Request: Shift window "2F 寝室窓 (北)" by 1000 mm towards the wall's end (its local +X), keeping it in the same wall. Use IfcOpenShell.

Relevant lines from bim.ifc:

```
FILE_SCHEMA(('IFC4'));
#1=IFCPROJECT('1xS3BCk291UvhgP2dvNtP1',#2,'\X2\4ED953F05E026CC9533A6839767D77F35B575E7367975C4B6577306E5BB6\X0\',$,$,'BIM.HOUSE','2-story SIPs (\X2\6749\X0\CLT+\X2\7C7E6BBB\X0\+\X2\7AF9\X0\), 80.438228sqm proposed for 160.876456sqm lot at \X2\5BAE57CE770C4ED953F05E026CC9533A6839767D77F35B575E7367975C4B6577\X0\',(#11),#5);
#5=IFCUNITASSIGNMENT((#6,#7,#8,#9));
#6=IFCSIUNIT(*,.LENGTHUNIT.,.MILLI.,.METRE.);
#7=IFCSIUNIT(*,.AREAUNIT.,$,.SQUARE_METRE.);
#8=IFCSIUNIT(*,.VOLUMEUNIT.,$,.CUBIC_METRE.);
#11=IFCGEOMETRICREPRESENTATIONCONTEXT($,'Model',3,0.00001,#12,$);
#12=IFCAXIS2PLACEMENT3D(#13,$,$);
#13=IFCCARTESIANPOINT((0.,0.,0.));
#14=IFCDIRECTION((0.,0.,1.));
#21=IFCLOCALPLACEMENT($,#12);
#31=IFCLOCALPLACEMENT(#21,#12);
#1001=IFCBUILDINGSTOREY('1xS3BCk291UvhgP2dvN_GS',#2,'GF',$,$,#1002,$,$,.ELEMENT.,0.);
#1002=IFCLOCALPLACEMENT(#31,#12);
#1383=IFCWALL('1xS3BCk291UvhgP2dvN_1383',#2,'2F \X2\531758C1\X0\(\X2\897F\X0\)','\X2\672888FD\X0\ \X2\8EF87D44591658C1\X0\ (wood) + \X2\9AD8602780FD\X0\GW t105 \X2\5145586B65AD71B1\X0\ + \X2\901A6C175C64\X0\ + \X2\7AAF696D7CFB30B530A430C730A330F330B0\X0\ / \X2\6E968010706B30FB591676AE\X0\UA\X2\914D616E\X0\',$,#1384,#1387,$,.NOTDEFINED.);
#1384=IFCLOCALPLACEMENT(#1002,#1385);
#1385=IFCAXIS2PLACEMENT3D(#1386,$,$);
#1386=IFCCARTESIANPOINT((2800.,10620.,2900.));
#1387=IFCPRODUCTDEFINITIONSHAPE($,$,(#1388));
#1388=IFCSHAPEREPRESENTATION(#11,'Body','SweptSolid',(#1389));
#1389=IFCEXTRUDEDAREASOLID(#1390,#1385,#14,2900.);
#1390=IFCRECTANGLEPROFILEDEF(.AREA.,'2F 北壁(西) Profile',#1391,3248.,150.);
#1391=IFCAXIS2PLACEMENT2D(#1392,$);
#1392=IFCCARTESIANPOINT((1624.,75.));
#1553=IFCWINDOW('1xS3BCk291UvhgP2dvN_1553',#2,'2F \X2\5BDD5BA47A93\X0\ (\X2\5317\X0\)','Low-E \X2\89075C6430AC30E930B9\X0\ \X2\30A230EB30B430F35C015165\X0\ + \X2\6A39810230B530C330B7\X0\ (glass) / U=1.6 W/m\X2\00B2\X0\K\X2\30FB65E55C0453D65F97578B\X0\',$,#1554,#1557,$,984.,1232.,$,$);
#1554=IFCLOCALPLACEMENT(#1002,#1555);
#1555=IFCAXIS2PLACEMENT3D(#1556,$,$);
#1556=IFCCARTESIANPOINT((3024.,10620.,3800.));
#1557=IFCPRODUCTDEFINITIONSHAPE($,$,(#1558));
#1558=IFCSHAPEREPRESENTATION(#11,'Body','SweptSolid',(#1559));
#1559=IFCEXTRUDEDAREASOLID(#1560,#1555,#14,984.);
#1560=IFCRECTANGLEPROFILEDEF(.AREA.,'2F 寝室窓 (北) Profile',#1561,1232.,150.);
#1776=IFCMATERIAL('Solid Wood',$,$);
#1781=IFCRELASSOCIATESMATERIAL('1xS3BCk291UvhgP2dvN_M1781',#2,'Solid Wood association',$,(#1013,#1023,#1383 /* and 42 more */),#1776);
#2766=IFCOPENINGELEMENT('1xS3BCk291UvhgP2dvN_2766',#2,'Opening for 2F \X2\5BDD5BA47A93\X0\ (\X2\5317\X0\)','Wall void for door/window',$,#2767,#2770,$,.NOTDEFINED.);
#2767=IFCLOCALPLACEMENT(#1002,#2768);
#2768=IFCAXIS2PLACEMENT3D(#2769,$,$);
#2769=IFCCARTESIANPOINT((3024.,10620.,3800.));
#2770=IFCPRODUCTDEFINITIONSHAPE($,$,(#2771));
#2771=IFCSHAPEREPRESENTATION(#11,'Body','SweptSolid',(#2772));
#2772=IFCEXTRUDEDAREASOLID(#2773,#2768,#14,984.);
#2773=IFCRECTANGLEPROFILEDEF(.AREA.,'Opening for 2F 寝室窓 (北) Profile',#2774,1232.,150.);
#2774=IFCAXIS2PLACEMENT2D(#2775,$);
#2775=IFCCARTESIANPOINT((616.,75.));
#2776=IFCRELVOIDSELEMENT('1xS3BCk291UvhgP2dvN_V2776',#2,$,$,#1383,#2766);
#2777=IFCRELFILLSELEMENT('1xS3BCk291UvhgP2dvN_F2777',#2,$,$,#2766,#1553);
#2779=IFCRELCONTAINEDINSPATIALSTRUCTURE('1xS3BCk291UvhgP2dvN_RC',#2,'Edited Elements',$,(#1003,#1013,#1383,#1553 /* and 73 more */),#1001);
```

```python
import ifcopenshell
import ifcopenshell.api.geometry
import ifcopenshell.util.placement

model = ifcopenshell.open("bim.ifc")

window = model.by_guid("1xS3BCk291UvhgP2dvN_1553")
opening = window.FillsVoids[0].RelatingOpeningElement
wall = opening.VoidsElements[0].RelatingBuildingElement

wall_matrix = ifcopenshell.util.placement.get_local_placement(wall.ObjectPlacement)
shift = wall_matrix[:3, 0] * 1000.0
before = ifcopenshell.util.placement.get_local_placement(window.ObjectPlacement)[:3, 3].copy()

# The window is not placed relative to its opening, so move both.
for product in (opening, window):
    matrix = ifcopenshell.util.placement.get_local_placement(product.ObjectPlacement)
    matrix[:3, 3] += shift
    ifcopenshell.api.geometry.edit_object_placement(model, product=product, matrix=matrix, is_si=False)

after = ifcopenshell.util.placement.get_local_placement(window.ObjectPlacement)[:3, 3]
print("window moved by", (after - before).round(3) + 0.0)

model.write("bim_rev.ifc")
```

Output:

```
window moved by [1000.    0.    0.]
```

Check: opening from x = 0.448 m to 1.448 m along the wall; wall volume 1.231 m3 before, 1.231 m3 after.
